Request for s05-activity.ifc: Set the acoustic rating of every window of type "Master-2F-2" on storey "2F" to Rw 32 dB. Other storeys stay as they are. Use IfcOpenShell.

First a look at what the model holds.

```python
import ifcopenshell
import ifcopenshell.util.element

model = ifcopenshell.open("s05-activity.ifc")
print(model.schema)
storey = next(s for s in model.by_type("IfcBuildingStorey") if s.Name == "2F")
windows = [e for e in ifcopenshell.util.element.get_decomposition(storey) if e.is_a("IfcWindow")]
seen = {}
for e in windows:
    element_type = ifcopenshell.util.element.get_type(e)
    key = (element_type.Name if element_type != e and element_type else None, ifcopenshell.util.element.get_pset(e, "Pset_WindowCommon", "AcousticRating"))
    seen[key] = seen.get(key, 0) + 1
for (name, value), count in sorted(seen.items(), key=str):
    print(count, "x", name, "|", value)
```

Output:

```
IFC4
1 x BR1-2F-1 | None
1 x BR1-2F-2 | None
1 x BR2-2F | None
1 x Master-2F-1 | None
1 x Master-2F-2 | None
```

```python
import ifcopenshell
import ifcopenshell.api.pset
import ifcopenshell.util.element

model = ifcopenshell.open("s05-activity.ifc")

storey = next(s for s in model.by_type("IfcBuildingStorey") if s.Name == "2F")
windows = [e for e in ifcopenshell.util.element.get_decomposition(storey) if e.is_a("IfcWindow")]

count = 0
for e in windows:
    element_type = ifcopenshell.util.element.get_type(e)
    if element_type in (None, e) or element_type.Name != "Master-2F-2":
        continue
    # add_pset returns the element's existing set when there is one.
    pset = ifcopenshell.api.pset.add_pset(model, product=e, name="Pset_WindowCommon")
    ifcopenshell.api.pset.edit_pset(model, pset=pset, properties={"AcousticRating": "Rw 32 dB"})
    count += 1

print(count, "windows updated")

model.write("s05-activity-out.ifc")
```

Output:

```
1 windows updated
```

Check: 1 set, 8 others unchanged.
